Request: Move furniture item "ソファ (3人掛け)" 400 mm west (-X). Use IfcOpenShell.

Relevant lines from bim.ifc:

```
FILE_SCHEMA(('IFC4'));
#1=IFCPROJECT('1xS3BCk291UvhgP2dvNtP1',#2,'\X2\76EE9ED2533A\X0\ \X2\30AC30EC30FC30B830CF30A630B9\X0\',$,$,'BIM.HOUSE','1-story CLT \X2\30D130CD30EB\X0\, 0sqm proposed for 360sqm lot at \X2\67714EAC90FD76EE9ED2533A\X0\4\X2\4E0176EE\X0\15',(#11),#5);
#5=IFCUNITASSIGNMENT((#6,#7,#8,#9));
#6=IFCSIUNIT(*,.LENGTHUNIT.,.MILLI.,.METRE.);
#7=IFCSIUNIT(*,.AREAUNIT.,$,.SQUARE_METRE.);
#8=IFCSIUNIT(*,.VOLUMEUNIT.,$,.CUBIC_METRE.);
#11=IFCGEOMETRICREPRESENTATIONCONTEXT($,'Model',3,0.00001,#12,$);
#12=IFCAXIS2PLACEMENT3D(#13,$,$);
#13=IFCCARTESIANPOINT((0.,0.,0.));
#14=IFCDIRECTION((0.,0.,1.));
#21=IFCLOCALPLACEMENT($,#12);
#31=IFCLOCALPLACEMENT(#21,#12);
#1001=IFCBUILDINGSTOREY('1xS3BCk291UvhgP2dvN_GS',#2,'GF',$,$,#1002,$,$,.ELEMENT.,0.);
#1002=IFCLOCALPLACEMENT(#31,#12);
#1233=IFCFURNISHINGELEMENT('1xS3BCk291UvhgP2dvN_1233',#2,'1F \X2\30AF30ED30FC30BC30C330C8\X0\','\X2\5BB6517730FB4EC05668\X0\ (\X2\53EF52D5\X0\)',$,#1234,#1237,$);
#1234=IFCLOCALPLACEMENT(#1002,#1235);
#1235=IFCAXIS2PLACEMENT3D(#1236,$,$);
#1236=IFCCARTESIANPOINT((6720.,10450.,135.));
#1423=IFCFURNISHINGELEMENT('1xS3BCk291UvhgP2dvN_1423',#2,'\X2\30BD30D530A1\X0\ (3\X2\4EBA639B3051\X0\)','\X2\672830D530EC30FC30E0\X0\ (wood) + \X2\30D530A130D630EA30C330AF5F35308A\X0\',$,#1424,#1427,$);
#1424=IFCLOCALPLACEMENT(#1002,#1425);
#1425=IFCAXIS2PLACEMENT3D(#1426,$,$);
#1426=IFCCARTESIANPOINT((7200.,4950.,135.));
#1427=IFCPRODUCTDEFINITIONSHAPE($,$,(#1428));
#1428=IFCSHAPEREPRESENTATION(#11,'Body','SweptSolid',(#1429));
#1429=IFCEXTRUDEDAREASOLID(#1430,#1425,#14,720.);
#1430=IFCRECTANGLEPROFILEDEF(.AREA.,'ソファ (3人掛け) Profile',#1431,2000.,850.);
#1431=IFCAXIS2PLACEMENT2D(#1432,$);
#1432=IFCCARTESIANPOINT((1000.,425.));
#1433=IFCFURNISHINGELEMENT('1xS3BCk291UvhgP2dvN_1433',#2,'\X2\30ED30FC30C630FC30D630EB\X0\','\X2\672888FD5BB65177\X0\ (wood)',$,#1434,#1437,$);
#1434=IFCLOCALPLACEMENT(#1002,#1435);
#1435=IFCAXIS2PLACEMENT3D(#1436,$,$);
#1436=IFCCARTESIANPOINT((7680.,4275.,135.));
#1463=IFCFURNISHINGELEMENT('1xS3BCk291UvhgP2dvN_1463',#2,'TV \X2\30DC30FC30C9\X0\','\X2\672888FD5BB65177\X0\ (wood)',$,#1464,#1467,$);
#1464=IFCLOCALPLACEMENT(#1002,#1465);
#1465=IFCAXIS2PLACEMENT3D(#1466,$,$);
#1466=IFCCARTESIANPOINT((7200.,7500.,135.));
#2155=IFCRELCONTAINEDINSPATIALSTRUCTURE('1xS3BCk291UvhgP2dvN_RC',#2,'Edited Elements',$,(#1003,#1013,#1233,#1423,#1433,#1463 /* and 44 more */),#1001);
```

```python
import ifcopenshell
import ifcopenshell.api.geometry
import ifcopenshell.util.placement

model = ifcopenshell.open("bim.ifc")

item = model.by_id(1423)
matrix = ifcopenshell.util.placement.get_local_placement(item.ObjectPlacement)
matrix[0, 3] -= 400.0
ifcopenshell.api.geometry.edit_object_placement(model, product=item, matrix=matrix, is_si=False)

print(ifcopenshell.util.placement.get_local_placement(item.ObjectPlacement).round(3) + 0.0)

model.write("bim_rev.ifc")
```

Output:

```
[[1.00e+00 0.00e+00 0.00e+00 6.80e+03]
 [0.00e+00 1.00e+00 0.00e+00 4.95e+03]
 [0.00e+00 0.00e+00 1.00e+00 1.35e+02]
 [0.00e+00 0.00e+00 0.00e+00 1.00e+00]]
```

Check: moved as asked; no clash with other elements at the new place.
